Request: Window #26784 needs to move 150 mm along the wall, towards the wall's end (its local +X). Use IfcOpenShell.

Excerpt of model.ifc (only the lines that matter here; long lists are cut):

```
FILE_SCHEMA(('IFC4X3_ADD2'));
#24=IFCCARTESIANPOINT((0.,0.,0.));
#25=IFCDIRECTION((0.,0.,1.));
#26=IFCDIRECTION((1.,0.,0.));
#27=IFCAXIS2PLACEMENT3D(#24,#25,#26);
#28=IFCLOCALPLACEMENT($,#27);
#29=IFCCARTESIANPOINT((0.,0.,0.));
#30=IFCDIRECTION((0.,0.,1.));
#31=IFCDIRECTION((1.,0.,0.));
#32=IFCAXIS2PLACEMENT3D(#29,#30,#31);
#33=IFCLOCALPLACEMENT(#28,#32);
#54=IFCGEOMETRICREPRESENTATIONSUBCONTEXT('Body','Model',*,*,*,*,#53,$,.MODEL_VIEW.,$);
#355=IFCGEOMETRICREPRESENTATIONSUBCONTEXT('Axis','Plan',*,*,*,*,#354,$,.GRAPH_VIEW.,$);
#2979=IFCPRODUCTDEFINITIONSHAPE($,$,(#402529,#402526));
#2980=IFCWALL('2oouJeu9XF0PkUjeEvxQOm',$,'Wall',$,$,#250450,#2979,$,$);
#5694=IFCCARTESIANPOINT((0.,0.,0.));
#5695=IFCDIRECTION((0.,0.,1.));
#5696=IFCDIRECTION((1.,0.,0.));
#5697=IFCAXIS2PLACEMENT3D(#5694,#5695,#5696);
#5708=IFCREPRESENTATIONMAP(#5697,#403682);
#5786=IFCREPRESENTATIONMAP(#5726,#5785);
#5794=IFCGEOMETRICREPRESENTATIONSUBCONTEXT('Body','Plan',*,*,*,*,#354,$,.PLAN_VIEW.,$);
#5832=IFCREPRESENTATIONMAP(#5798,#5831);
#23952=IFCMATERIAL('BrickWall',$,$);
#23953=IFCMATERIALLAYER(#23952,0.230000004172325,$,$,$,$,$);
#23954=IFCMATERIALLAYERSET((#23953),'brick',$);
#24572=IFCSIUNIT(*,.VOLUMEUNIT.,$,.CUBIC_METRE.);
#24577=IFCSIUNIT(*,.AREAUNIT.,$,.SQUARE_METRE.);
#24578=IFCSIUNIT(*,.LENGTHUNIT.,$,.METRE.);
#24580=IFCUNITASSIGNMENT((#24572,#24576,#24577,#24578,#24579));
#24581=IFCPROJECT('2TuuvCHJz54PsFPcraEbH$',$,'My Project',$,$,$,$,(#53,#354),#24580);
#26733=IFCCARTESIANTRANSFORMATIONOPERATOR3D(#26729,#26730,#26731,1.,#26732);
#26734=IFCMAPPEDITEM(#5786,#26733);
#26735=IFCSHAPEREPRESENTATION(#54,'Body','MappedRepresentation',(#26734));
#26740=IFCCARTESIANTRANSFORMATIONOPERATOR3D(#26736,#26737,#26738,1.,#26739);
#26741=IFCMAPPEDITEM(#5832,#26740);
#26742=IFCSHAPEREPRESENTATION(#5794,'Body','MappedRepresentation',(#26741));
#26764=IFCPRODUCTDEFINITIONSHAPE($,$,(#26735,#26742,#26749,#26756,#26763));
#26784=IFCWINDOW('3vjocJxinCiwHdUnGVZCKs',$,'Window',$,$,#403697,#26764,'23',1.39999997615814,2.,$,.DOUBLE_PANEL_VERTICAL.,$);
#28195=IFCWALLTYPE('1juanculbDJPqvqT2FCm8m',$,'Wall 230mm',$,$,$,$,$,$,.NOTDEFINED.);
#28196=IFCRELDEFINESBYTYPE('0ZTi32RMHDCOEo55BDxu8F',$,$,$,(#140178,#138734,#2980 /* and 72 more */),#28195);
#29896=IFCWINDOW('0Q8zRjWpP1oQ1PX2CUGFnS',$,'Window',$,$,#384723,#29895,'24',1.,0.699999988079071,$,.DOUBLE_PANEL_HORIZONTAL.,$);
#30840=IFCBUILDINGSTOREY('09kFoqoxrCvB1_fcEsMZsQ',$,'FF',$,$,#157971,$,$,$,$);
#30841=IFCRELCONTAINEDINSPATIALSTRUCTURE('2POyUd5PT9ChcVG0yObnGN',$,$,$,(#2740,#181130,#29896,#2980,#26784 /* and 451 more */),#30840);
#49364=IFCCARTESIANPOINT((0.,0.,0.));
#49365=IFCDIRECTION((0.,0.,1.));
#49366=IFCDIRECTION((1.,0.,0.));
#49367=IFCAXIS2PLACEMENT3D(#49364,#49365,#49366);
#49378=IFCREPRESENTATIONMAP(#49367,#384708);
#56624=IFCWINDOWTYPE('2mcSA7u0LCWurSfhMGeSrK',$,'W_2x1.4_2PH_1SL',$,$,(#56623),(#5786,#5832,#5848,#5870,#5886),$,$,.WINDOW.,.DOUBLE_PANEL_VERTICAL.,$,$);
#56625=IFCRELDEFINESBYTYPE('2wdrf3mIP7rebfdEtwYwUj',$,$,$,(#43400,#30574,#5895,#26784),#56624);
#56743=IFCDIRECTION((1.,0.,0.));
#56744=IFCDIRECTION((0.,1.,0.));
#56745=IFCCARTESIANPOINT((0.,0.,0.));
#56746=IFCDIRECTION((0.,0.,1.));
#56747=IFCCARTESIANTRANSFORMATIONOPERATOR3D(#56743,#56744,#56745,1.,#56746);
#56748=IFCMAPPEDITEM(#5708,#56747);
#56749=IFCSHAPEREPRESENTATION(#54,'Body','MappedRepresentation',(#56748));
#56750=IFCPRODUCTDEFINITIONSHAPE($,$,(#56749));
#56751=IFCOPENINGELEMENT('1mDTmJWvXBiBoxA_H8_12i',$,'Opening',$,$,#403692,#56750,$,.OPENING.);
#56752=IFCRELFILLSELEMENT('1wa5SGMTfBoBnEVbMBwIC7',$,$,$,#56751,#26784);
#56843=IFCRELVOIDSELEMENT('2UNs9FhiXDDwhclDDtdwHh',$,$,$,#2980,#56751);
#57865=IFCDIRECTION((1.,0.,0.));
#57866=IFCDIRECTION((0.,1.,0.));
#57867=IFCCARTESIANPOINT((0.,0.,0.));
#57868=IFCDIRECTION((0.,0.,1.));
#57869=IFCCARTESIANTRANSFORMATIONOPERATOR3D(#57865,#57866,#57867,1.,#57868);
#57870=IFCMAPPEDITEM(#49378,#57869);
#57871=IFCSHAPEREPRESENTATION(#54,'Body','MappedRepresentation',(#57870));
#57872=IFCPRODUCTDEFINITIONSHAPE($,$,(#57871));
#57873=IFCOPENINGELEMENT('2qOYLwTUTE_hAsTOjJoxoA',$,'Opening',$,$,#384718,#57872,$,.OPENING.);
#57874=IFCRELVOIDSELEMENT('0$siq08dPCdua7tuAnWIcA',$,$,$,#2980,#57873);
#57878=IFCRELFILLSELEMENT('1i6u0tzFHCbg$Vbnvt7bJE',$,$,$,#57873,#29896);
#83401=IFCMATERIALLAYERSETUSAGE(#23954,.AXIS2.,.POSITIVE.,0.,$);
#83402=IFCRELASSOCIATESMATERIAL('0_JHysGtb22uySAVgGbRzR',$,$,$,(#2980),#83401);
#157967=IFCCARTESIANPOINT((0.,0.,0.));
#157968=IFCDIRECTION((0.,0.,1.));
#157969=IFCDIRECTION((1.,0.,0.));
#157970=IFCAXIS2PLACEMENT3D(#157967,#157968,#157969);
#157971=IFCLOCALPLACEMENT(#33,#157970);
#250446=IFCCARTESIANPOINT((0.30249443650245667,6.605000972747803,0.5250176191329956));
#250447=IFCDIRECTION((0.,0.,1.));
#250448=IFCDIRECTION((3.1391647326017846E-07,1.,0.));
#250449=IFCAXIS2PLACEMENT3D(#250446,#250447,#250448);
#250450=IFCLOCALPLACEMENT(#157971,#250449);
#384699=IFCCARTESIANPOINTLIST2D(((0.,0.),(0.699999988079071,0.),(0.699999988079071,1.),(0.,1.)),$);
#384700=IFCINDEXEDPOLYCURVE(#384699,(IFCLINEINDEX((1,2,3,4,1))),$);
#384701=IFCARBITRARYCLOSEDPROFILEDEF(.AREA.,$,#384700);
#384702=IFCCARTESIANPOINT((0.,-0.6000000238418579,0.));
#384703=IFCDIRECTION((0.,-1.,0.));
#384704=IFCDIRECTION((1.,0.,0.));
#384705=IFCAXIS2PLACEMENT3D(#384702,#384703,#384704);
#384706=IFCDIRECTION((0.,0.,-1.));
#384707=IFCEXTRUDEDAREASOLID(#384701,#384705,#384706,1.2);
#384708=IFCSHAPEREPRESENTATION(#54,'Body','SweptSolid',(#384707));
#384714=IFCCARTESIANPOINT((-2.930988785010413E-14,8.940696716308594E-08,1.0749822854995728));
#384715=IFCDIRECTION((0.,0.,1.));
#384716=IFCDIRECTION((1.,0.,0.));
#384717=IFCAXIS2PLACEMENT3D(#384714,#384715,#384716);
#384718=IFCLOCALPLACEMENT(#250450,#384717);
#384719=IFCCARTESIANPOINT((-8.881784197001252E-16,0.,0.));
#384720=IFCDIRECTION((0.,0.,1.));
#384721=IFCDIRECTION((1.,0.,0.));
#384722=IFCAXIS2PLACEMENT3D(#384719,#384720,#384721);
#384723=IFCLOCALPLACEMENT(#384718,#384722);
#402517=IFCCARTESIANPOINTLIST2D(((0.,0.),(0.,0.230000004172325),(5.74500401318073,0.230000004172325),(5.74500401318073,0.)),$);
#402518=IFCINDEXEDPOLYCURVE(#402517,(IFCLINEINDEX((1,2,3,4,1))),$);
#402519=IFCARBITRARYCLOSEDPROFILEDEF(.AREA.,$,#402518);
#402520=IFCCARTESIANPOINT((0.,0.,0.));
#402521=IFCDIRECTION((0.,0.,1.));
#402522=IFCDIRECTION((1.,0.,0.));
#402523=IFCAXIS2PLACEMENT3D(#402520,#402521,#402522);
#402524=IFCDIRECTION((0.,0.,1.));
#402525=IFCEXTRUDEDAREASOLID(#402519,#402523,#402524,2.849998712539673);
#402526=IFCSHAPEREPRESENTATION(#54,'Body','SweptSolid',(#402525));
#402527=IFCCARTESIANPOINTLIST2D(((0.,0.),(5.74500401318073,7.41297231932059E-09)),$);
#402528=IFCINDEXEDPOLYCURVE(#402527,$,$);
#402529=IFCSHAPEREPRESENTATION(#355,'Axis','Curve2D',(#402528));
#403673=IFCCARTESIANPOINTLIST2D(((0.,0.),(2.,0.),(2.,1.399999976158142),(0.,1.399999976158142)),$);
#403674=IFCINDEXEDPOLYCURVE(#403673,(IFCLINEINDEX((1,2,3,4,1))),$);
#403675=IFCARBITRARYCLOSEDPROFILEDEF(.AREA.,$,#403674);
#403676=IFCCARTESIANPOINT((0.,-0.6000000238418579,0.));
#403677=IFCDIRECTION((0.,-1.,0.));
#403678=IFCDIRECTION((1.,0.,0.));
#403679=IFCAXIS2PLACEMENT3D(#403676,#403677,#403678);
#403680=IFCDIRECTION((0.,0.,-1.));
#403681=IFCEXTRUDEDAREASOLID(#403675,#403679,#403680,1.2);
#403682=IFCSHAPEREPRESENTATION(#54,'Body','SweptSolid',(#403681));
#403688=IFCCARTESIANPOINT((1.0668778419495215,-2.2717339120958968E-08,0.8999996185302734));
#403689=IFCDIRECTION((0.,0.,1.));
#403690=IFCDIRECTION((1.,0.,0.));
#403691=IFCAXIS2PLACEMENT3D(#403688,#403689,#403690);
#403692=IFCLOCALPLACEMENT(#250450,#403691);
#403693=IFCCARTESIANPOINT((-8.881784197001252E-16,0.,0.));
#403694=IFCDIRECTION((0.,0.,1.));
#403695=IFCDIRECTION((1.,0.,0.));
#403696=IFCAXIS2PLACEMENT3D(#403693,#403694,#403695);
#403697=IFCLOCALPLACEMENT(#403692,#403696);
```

```python
import ifcopenshell
import ifcopenshell.api.geometry
import ifcopenshell.util.placement
import ifcopenshell.util.unit

model = ifcopenshell.open("model.ifc")
unit_scale = ifcopenshell.util.unit.calculate_unit_scale(model)

window = model.by_guid("3vjocJxinCiwHdUnGVZCKs")
opening = window.FillsVoids[0].RelatingOpeningElement
wall = opening.VoidsElements[0].RelatingBuildingElement

wall_matrix = ifcopenshell.util.placement.get_local_placement(wall.ObjectPlacement)
shift = wall_matrix[:3, 0] * 0.15 / unit_scale
before = ifcopenshell.util.placement.get_local_placement(window.ObjectPlacement)[:3, 3].copy()

# The window is placed relative to its opening, so it follows when the opening moves.
matrix = ifcopenshell.util.placement.get_local_placement(opening.ObjectPlacement)
matrix[:3, 3] += shift
ifcopenshell.api.geometry.edit_object_placement(
    model, product=opening, matrix=matrix, is_si=False, should_transform_children=True
)

after = ifcopenshell.util.placement.get_local_placement(window.ObjectPlacement)[:3, 3]
print("window moved by", (after - before).round(3) + 0.0)

model.write("model_updated.ifc")
```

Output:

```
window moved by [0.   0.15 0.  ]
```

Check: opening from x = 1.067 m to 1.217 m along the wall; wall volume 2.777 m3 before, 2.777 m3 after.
